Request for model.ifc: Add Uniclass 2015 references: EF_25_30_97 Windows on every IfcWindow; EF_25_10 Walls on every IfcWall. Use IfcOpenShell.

First a look at what the model holds.

```python
import ifcopenshell

model = ifcopenshell.open("model.ifc")
print(model.schema)
print("classifications:", [c.Name for c in model.by_type("IfcClassification")])
for ifc_class in ("IfcDoor", "IfcRoof", "IfcStair", "IfcWall", "IfcWindow"):
    print(ifc_class, len(model.by_type(ifc_class)))
```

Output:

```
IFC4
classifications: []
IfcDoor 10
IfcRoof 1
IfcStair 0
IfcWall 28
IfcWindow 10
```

```python
import ifcopenshell
import ifcopenshell.api.classification

model = ifcopenshell.open("model.ifc")

system = ifcopenshell.api.classification.add_classification(model, classification="Uniclass 2015")

codes = {
    "IfcWindow": ("EF_25_30_97", "Windows"),
    "IfcWall": ("EF_25_10", "Walls"),
}
for ifc_class, (code, name) in codes.items():
    products = model.by_type(ifc_class)
    ifcopenshell.api.classification.add_reference(
        model, products=products, classification=system, identification=code, name=name
    )
    print(code, len(products))

model.write("model_edited.ifc")
```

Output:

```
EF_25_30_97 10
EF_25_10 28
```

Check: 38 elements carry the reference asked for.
